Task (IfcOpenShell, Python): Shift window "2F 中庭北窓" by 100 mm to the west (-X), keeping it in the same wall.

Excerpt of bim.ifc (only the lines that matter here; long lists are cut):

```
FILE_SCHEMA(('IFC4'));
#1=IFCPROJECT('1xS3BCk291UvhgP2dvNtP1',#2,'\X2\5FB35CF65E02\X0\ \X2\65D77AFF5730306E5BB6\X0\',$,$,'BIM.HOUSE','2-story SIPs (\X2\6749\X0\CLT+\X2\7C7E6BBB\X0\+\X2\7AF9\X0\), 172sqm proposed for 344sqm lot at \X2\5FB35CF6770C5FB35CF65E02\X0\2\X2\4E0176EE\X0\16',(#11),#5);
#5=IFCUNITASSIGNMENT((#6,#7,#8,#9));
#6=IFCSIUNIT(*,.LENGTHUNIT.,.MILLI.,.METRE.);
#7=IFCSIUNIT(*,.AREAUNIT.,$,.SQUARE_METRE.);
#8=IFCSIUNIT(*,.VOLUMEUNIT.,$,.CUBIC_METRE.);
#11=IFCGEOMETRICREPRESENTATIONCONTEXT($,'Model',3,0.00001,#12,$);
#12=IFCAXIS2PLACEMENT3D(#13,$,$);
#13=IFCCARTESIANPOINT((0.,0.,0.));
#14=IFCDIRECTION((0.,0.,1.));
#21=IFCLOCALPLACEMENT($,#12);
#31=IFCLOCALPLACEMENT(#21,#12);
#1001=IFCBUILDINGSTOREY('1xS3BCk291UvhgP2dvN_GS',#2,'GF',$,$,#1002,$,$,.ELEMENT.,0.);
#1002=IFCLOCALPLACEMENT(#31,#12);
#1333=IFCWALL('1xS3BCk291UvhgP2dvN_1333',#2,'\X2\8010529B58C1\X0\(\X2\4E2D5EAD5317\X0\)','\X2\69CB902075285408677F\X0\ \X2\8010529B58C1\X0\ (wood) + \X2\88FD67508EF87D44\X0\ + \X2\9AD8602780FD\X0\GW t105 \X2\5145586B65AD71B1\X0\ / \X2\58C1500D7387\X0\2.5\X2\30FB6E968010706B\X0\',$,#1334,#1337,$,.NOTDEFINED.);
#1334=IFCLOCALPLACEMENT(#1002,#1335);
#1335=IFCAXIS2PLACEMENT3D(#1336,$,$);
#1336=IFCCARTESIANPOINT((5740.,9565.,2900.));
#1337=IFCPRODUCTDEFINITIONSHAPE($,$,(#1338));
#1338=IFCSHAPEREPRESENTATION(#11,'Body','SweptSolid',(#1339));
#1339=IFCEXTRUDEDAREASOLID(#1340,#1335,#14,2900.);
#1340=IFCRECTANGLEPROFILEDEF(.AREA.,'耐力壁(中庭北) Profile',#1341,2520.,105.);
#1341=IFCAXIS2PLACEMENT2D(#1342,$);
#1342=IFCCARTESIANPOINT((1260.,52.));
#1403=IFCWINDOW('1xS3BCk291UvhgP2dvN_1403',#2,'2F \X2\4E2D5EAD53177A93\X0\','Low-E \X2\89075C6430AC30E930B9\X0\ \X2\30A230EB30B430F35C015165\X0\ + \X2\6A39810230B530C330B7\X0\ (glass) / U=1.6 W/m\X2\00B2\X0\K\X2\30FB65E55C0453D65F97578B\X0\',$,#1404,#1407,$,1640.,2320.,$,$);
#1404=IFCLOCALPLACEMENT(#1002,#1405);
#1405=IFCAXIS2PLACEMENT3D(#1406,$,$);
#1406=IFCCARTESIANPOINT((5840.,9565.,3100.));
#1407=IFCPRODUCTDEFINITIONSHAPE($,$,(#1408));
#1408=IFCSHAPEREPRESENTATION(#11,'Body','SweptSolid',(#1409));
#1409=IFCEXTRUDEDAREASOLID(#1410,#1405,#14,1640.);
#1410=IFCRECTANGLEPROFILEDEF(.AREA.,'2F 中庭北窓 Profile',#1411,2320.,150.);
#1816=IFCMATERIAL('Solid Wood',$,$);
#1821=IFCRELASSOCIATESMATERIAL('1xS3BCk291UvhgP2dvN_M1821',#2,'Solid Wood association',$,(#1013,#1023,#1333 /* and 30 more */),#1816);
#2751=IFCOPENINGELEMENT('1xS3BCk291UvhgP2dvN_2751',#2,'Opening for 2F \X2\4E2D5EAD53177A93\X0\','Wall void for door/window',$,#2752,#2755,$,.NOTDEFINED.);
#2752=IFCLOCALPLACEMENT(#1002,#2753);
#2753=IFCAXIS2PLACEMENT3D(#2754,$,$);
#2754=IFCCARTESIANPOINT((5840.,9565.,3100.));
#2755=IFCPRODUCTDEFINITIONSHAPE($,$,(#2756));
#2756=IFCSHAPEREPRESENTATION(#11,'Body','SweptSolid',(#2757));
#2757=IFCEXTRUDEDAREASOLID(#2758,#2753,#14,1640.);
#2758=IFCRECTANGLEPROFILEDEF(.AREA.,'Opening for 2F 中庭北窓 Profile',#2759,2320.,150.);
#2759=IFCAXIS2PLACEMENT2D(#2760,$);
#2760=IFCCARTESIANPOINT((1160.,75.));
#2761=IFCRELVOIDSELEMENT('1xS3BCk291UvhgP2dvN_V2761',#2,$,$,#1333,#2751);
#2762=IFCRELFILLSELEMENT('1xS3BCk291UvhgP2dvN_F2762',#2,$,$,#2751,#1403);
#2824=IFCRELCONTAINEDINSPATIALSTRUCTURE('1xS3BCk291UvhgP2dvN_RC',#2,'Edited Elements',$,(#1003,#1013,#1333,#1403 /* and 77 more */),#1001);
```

```python
import ifcopenshell
import ifcopenshell.api.geometry
import ifcopenshell.util.placement
import ifcopenshell.util.unit

model = ifcopenshell.open("bim.ifc")
unit_scale = ifcopenshell.util.unit.calculate_unit_scale(model)

window = model.by_guid("1xS3BCk291UvhgP2dvN_1403")
opening = window.FillsVoids[0].RelatingOpeningElement
wall = opening.VoidsElements[0].RelatingBuildingElement

wall_matrix = ifcopenshell.util.placement.get_local_placement(wall.ObjectPlacement)
shift = wall_matrix[:3, 0] * -0.1 / unit_scale
before = ifcopenshell.util.placement.get_local_placement(window.ObjectPlacement)[:3, 3].copy()

# The window is not placed relative to its opening, so move both.
for product in (opening, window):
    matrix = ifcopenshell.util.placement.get_local_placement(product.ObjectPlacement)
    matrix[:3, 3] += shift
    ifcopenshell.api.geometry.edit_object_placement(model, product=product, matrix=matrix, is_si=False)

after = ifcopenshell.util.placement.get_local_placement(window.ObjectPlacement)[:3, 3]
print("window moved by", (after - before).round(3) + 0.0)

model.write("bim-out.ifc")
```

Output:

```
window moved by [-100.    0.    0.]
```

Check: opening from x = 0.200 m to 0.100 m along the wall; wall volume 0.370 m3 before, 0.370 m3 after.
